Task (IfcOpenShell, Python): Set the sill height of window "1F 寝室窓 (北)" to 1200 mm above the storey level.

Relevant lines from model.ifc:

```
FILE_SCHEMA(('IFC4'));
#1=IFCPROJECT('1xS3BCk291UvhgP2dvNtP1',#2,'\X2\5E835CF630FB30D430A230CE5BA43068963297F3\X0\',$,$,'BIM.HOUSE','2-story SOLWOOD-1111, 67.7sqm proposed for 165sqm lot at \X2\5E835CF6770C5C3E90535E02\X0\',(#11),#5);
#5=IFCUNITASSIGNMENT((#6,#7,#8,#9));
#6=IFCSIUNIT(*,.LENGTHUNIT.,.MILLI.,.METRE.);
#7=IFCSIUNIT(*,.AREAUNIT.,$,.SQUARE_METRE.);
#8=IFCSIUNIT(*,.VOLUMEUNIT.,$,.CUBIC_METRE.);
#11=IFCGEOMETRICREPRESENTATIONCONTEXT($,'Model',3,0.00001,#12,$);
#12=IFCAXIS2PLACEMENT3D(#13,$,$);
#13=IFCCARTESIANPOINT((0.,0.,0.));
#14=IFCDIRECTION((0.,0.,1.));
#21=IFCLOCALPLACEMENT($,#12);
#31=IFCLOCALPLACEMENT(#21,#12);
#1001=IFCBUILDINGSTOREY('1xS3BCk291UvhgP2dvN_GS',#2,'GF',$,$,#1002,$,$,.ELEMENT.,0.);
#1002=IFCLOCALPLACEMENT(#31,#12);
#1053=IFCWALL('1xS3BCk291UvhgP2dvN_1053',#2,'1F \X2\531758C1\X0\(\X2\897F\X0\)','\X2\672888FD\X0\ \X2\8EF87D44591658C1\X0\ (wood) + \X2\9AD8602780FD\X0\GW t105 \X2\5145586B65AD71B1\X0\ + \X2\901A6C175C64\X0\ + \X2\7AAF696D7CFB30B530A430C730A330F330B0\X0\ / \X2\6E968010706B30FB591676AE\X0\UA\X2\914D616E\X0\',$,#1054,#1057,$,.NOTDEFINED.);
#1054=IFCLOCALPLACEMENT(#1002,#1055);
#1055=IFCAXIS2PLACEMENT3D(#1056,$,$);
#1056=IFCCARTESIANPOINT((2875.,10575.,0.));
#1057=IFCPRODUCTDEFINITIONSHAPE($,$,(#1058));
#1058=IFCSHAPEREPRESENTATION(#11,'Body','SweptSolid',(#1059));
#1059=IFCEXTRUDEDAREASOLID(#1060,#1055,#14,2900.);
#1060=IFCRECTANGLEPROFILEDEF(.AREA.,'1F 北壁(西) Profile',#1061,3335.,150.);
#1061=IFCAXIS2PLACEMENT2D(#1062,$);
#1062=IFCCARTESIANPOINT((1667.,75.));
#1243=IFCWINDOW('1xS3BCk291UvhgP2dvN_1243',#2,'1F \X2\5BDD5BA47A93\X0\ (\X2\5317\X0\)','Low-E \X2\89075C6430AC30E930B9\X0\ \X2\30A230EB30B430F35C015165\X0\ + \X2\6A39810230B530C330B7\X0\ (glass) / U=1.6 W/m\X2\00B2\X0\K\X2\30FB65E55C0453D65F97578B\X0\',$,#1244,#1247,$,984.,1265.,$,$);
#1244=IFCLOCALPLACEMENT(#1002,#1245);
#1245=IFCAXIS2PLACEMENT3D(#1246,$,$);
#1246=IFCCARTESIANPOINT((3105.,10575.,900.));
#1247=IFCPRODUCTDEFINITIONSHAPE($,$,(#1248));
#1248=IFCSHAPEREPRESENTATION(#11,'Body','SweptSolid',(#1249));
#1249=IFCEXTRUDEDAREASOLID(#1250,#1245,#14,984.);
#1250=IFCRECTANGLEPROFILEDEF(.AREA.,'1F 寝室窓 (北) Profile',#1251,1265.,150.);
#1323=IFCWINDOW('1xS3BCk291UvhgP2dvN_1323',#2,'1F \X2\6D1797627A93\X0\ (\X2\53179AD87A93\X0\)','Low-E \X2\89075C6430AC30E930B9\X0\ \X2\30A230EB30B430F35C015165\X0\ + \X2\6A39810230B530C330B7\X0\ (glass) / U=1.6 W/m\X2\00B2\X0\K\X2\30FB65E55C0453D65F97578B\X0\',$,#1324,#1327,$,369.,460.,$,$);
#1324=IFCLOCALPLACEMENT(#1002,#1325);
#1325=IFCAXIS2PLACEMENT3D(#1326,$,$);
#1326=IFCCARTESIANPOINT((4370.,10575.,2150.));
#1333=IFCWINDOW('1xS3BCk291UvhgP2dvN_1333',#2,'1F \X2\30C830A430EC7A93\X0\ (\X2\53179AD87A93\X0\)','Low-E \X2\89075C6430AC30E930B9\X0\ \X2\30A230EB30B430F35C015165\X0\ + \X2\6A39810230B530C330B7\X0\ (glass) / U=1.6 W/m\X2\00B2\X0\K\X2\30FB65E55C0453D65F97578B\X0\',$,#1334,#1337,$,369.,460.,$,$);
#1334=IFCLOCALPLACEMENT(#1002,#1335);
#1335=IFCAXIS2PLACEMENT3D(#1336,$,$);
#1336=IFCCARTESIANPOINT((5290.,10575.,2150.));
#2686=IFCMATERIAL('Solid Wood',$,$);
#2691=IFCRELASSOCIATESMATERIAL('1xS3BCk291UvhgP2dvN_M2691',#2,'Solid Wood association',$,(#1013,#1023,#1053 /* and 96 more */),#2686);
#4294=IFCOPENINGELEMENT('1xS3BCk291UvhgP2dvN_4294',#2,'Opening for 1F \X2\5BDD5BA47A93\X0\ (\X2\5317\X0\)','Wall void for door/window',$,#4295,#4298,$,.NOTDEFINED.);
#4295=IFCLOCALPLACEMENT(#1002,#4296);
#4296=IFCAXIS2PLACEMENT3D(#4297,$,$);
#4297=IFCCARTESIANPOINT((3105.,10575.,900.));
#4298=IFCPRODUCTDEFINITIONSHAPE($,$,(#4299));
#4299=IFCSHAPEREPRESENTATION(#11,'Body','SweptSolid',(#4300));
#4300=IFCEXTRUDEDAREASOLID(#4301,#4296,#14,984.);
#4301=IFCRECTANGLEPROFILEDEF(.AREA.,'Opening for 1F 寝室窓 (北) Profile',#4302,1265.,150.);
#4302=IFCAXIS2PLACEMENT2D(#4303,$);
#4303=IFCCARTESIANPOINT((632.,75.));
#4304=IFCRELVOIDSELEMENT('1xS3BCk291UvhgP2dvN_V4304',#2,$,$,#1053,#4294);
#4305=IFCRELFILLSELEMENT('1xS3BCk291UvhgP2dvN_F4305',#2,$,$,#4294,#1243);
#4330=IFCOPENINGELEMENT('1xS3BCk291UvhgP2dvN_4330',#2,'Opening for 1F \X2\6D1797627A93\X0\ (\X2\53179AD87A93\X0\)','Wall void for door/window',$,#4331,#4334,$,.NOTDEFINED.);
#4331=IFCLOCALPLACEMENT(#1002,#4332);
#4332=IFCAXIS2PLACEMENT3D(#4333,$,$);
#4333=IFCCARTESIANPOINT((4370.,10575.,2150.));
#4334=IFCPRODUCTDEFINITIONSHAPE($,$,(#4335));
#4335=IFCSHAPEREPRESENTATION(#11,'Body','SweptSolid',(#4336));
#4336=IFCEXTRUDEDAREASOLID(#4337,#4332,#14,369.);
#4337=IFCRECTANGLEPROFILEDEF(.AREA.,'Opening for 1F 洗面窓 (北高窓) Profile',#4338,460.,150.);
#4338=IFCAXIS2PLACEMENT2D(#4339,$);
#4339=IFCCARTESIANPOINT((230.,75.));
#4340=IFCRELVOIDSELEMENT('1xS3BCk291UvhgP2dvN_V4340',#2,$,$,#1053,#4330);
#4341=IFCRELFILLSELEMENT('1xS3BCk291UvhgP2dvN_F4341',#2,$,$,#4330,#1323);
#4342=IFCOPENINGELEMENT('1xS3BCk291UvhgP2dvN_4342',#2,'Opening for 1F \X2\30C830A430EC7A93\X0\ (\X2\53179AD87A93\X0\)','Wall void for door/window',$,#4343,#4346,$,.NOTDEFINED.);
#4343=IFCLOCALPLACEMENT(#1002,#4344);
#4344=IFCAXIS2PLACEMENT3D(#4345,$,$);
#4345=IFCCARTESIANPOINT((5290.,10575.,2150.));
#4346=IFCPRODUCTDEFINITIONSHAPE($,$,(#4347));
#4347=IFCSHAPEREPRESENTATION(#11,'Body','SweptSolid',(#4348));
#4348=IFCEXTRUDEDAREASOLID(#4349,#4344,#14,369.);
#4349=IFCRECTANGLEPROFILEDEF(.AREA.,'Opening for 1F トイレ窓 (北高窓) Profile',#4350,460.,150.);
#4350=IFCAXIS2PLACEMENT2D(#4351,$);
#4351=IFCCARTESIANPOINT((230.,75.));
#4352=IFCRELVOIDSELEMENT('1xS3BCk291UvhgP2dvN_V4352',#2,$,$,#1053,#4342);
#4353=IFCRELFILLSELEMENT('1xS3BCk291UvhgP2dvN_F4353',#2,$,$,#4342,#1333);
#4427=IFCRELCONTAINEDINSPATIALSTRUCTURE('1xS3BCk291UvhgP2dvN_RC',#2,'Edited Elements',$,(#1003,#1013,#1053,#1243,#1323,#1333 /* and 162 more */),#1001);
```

```python
import numpy as np
import ifcopenshell
import ifcopenshell.api.geometry
import ifcopenshell.geom
import ifcopenshell.util.element
import ifcopenshell.util.placement
import ifcopenshell.util.shape
import ifcopenshell.util.unit

model = ifcopenshell.open("model.ifc")
unit_scale = ifcopenshell.util.unit.calculate_unit_scale(model)

window = model.by_guid("1xS3BCk291UvhgP2dvN_1243")
opening = window.FillsVoids[0].RelatingOpeningElement
storey = ifcopenshell.util.element.get_container(window, ifc_class="IfcBuildingStorey")
level = ifcopenshell.util.placement.get_local_placement(storey.ObjectPlacement)[2, 3]

# The opening's origin need not be at the sill, so measure its lowest point.
shape = ifcopenshell.geom.create_shape(ifcopenshell.geom.settings(), opening)
bottom = ifcopenshell.util.shape.get_shape_bottom_elevation(shape, shape.geometry) / unit_scale
dz = level + 1.2 / unit_scale - bottom

shift = np.array([0.0, 0.0, dz])
# The window is not placed relative to its opening, so move both.
for product in (opening, window):
    matrix = ifcopenshell.util.placement.get_local_placement(product.ObjectPlacement)
    matrix[:3, 3] += shift
    ifcopenshell.api.geometry.edit_object_placement(model, product=product, matrix=matrix, is_si=False)

print(f"moved by {dz * unit_scale:+.3f} m")

model.write("model_edited.ifc")
```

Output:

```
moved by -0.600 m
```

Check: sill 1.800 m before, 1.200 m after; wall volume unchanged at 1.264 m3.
